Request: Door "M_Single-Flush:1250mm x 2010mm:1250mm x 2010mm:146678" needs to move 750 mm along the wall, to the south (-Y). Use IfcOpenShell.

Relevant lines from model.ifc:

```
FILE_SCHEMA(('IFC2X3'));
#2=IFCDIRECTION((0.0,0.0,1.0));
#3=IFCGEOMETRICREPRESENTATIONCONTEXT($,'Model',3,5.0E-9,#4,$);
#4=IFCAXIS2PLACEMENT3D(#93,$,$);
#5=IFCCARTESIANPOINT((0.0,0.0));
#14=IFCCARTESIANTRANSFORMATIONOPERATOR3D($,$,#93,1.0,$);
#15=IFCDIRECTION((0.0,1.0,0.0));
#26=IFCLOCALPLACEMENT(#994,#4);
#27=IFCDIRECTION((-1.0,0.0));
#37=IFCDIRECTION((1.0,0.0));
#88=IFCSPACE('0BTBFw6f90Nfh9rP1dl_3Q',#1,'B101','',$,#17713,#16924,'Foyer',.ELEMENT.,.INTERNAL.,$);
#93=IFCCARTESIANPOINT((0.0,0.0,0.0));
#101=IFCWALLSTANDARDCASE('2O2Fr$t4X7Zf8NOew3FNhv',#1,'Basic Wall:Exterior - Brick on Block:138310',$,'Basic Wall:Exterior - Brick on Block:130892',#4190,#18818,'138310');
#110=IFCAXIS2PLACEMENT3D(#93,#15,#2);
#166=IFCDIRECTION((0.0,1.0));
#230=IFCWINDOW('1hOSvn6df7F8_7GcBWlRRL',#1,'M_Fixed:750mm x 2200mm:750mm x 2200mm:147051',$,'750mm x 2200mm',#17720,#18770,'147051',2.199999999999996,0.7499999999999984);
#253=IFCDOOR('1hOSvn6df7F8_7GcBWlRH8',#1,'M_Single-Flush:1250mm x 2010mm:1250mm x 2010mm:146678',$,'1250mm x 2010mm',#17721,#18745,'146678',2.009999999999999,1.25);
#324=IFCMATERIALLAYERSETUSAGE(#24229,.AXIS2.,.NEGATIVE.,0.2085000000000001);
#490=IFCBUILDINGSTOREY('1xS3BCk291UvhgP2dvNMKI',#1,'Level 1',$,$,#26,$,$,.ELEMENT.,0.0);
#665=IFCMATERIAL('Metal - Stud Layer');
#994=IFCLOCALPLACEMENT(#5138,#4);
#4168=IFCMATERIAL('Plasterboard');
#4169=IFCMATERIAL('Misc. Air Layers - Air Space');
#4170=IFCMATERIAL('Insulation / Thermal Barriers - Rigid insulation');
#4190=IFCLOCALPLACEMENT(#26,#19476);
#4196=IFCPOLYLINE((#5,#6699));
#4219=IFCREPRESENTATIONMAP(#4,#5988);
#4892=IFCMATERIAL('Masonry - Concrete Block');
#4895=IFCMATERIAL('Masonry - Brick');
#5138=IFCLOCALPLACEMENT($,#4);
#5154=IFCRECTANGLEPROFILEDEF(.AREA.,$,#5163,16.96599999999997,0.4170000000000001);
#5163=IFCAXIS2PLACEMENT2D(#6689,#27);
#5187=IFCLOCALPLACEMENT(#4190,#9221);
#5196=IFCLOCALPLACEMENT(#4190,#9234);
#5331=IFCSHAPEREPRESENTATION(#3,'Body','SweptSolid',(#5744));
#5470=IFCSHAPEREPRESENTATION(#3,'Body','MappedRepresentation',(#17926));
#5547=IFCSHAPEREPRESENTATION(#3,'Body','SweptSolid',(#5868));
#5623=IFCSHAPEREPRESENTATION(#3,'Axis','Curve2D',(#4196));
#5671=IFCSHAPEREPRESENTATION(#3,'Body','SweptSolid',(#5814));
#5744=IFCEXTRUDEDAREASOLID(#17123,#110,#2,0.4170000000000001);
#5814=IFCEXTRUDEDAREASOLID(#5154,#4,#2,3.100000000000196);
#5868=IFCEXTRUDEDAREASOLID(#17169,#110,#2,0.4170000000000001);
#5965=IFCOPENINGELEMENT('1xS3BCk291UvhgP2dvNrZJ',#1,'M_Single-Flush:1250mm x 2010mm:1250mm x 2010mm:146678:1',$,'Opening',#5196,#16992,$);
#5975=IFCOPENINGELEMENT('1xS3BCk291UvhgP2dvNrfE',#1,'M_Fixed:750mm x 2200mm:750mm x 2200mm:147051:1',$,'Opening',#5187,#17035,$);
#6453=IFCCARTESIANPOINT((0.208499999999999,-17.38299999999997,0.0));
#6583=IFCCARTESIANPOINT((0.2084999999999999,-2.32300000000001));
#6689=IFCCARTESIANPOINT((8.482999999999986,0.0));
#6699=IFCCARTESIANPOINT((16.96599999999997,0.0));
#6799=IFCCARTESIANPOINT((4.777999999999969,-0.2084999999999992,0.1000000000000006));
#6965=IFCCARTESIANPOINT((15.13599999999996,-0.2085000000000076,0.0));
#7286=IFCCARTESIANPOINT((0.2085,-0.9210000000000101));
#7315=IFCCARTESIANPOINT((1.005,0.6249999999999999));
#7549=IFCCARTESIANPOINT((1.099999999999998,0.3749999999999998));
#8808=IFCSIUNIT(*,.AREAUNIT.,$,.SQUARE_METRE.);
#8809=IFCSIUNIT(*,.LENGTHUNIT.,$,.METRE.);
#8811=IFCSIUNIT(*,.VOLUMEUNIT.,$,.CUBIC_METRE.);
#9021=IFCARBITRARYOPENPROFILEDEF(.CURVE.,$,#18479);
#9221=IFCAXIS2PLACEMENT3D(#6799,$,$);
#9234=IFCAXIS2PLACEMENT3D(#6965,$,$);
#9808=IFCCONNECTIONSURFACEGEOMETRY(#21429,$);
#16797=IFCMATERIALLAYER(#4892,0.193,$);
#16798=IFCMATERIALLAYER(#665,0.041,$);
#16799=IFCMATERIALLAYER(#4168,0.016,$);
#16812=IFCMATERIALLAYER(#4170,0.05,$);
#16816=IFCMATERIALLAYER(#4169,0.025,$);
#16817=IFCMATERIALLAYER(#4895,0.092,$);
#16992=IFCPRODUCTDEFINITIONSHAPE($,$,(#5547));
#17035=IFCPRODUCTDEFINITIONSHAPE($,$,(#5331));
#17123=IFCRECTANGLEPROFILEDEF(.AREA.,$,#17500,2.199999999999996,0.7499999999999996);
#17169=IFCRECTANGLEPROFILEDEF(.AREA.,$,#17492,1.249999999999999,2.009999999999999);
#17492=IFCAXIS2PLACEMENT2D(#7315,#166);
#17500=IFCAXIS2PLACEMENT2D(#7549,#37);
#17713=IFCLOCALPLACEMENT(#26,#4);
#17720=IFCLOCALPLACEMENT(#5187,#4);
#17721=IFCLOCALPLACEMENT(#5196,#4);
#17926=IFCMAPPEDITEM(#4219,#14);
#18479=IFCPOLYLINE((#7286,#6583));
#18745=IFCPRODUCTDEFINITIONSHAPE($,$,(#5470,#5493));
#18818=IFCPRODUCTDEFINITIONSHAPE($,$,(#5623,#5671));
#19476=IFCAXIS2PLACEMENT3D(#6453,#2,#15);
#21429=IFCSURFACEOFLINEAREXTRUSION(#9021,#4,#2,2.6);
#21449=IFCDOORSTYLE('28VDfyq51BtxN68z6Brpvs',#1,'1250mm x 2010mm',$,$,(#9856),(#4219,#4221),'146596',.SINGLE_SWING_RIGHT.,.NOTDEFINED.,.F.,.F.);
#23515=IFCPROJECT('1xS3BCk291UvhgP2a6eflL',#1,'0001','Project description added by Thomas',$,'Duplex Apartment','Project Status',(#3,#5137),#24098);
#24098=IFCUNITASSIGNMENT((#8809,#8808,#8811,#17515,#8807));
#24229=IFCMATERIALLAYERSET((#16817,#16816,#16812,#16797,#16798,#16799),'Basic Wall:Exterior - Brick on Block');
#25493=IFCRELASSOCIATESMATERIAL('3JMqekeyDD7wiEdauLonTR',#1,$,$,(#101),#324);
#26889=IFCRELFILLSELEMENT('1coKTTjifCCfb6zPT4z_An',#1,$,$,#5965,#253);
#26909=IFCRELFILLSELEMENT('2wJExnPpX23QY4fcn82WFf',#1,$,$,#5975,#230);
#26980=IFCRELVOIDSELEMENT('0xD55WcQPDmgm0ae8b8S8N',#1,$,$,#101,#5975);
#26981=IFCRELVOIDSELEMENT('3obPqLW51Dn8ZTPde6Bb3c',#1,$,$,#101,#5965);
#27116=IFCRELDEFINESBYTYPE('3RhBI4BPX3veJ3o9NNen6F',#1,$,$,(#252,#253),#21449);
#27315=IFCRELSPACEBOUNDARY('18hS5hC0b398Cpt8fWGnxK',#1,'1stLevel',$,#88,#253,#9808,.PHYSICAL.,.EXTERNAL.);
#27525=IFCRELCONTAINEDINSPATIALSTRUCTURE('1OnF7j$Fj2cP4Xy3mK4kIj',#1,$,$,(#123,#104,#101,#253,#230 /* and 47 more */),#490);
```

```python
import numpy as np
import ifcopenshell
import ifcopenshell.api.geometry
import ifcopenshell.util.placement

model = ifcopenshell.open("model.ifc")

door = model.by_guid("1hOSvn6df7F8_7GcBWlRH8")
opening = door.FillsVoids[0].RelatingOpeningElement
wall = opening.VoidsElements[0].RelatingBuildingElement

wall_matrix = ifcopenshell.util.placement.get_local_placement(wall.ObjectPlacement)
shift = wall_matrix[:3, 0] * -0.75
before = ifcopenshell.util.placement.get_local_placement(door.ObjectPlacement)[:3, 3].copy()

# The door is placed relative to its opening, so it follows when the opening moves.
matrix = ifcopenshell.util.placement.get_local_placement(opening.ObjectPlacement)
matrix[:3, 3] += shift
ifcopenshell.api.geometry.edit_object_placement(
    model, product=opening, matrix=matrix, is_si=False, should_transform_children=True
)

# Space boundary surfaces are stored in each space's coordinates; move them too.
for rel in door.ProvidesBoundaries:
    if not rel.ConnectionGeometry:
        continue
    surface = rel.ConnectionGeometry.SurfaceOnRelatingElement
    space_matrix = ifcopenshell.util.placement.get_local_placement(rel.RelatingSpace.ObjectPlacement)
    point = np.array(surface.Position.Location.Coordinates) + space_matrix[:3, :3].T @ shift
    surface.Position = model.createIfcAxis2Placement3D(
        model.createIfcCartesianPoint(point.tolist()), surface.Position.Axis, surface.Position.RefDirection
    )

after = ifcopenshell.util.placement.get_local_placement(door.ObjectPlacement)[:3, 3]
print("door moved by", (after - before).round(3) + 0.0)

model.write("model_v2.ifc")
```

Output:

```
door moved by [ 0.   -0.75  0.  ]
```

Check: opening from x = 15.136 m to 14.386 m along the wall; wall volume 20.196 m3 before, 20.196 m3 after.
